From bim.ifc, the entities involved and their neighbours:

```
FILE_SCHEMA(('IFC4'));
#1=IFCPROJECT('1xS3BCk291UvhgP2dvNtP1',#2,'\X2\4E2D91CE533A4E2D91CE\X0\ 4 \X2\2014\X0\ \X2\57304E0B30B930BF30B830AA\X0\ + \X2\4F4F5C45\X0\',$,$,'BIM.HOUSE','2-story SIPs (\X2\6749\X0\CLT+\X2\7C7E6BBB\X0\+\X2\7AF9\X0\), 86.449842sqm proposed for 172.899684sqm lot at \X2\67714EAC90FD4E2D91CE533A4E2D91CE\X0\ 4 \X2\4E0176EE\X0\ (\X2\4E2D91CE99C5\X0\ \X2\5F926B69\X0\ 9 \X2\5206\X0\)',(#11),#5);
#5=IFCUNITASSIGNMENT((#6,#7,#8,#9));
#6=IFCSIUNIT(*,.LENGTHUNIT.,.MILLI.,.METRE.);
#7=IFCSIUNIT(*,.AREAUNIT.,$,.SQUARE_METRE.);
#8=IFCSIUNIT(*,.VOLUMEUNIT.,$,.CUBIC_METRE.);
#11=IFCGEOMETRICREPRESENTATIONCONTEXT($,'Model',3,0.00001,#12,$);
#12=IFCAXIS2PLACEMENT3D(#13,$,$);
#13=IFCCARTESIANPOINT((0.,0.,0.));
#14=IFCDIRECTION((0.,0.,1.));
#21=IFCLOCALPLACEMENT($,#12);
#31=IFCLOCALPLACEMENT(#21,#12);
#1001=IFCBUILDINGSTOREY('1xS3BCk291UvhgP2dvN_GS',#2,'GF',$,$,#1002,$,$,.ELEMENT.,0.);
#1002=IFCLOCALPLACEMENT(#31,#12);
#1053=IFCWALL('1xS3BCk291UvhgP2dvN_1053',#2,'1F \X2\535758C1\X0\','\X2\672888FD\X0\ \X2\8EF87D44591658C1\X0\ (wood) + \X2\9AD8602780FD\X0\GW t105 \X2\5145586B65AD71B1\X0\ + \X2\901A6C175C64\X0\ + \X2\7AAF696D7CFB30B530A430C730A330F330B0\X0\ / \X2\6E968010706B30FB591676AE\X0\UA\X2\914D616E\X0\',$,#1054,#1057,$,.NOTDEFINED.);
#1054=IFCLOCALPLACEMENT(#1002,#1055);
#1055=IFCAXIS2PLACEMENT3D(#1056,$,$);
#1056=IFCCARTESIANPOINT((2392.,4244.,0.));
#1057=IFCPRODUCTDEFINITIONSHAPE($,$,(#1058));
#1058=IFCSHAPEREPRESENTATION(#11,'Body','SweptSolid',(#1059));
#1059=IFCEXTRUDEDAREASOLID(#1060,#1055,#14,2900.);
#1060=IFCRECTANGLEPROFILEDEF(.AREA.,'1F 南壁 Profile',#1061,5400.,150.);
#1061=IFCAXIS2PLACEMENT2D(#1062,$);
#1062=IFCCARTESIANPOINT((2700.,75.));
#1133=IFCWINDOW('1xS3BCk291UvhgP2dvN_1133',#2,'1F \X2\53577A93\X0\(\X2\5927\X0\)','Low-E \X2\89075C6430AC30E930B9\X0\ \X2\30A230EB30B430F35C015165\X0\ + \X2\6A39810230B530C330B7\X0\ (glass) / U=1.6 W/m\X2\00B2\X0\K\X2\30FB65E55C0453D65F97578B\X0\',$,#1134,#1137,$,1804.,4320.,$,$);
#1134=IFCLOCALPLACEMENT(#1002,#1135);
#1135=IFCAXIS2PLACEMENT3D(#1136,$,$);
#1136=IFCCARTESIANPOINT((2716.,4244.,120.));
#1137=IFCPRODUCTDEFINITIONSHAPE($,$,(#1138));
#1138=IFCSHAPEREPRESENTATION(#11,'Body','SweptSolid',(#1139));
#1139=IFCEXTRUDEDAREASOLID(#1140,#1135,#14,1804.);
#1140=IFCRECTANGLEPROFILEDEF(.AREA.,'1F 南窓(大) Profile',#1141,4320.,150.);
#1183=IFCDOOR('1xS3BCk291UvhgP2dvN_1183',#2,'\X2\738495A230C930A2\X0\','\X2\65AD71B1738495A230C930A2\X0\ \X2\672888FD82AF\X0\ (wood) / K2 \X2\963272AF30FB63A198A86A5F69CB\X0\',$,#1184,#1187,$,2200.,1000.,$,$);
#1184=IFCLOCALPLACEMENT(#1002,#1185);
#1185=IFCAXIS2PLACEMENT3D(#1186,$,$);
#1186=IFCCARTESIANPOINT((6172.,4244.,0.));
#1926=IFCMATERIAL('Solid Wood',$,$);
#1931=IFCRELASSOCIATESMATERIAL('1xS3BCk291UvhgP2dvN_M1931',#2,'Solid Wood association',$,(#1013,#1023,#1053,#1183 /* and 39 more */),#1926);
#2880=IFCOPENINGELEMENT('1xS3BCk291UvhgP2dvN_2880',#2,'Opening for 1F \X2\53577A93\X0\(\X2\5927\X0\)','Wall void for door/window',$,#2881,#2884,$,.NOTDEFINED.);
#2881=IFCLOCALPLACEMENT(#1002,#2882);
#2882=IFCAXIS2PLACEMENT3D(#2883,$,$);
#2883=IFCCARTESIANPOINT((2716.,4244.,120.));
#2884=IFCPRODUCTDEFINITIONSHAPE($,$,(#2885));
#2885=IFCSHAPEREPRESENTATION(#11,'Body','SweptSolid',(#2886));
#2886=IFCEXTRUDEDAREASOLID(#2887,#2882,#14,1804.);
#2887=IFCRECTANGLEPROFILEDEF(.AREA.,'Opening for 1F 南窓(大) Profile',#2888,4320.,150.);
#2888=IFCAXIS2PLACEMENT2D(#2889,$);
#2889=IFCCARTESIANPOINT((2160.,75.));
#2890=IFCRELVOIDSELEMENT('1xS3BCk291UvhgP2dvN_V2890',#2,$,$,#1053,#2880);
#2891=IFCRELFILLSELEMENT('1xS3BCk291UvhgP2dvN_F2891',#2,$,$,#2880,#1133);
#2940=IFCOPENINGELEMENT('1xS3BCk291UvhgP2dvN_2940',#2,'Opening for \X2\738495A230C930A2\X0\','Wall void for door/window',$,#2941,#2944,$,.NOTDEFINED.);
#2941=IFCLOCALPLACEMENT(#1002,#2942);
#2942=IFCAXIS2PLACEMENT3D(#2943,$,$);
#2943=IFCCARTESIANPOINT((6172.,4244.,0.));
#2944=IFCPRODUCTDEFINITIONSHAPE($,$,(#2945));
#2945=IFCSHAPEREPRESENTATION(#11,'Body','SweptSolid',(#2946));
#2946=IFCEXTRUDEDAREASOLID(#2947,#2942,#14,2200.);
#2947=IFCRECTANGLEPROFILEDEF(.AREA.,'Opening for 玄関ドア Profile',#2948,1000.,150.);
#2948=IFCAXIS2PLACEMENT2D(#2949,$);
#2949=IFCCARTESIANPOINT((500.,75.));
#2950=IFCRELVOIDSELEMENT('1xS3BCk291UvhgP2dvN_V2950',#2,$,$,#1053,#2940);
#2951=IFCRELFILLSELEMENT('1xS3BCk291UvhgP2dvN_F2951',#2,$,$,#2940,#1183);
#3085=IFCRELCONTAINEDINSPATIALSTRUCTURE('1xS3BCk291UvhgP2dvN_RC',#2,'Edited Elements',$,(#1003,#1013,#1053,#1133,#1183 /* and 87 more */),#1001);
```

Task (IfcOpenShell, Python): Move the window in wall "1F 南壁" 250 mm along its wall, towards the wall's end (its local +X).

```python
import ifcopenshell
import ifcopenshell.api.geometry
import ifcopenshell.util.placement
import ifcopenshell.util.unit

model = ifcopenshell.open("bim.ifc")
unit_scale = ifcopenshell.util.unit.calculate_unit_scale(model)

window = model.by_guid("1xS3BCk291UvhgP2dvN_1133")
opening = window.FillsVoids[0].RelatingOpeningElement
wall = opening.VoidsElements[0].RelatingBuildingElement

wall_matrix = ifcopenshell.util.placement.get_local_placement(wall.ObjectPlacement)
shift = wall_matrix[:3, 0] * 0.25 / unit_scale
before = ifcopenshell.util.placement.get_local_placement(window.ObjectPlacement)[:3, 3].copy()

# The window is not placed relative to its opening, so move both.
for product in (opening, window):
    matrix = ifcopenshell.util.placement.get_local_placement(product.ObjectPlacement)
    matrix[:3, 3] += shift
    ifcopenshell.api.geometry.edit_object_placement(model, product=product, matrix=matrix, is_si=False)

after = ifcopenshell.util.placement.get_local_placement(window.ObjectPlacement)[:3, 3]
print("window moved by", (after - before).round(3) + 0.0)

model.write("bim_rev.ifc")
```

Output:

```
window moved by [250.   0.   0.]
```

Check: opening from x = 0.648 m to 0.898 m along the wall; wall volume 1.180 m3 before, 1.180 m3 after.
